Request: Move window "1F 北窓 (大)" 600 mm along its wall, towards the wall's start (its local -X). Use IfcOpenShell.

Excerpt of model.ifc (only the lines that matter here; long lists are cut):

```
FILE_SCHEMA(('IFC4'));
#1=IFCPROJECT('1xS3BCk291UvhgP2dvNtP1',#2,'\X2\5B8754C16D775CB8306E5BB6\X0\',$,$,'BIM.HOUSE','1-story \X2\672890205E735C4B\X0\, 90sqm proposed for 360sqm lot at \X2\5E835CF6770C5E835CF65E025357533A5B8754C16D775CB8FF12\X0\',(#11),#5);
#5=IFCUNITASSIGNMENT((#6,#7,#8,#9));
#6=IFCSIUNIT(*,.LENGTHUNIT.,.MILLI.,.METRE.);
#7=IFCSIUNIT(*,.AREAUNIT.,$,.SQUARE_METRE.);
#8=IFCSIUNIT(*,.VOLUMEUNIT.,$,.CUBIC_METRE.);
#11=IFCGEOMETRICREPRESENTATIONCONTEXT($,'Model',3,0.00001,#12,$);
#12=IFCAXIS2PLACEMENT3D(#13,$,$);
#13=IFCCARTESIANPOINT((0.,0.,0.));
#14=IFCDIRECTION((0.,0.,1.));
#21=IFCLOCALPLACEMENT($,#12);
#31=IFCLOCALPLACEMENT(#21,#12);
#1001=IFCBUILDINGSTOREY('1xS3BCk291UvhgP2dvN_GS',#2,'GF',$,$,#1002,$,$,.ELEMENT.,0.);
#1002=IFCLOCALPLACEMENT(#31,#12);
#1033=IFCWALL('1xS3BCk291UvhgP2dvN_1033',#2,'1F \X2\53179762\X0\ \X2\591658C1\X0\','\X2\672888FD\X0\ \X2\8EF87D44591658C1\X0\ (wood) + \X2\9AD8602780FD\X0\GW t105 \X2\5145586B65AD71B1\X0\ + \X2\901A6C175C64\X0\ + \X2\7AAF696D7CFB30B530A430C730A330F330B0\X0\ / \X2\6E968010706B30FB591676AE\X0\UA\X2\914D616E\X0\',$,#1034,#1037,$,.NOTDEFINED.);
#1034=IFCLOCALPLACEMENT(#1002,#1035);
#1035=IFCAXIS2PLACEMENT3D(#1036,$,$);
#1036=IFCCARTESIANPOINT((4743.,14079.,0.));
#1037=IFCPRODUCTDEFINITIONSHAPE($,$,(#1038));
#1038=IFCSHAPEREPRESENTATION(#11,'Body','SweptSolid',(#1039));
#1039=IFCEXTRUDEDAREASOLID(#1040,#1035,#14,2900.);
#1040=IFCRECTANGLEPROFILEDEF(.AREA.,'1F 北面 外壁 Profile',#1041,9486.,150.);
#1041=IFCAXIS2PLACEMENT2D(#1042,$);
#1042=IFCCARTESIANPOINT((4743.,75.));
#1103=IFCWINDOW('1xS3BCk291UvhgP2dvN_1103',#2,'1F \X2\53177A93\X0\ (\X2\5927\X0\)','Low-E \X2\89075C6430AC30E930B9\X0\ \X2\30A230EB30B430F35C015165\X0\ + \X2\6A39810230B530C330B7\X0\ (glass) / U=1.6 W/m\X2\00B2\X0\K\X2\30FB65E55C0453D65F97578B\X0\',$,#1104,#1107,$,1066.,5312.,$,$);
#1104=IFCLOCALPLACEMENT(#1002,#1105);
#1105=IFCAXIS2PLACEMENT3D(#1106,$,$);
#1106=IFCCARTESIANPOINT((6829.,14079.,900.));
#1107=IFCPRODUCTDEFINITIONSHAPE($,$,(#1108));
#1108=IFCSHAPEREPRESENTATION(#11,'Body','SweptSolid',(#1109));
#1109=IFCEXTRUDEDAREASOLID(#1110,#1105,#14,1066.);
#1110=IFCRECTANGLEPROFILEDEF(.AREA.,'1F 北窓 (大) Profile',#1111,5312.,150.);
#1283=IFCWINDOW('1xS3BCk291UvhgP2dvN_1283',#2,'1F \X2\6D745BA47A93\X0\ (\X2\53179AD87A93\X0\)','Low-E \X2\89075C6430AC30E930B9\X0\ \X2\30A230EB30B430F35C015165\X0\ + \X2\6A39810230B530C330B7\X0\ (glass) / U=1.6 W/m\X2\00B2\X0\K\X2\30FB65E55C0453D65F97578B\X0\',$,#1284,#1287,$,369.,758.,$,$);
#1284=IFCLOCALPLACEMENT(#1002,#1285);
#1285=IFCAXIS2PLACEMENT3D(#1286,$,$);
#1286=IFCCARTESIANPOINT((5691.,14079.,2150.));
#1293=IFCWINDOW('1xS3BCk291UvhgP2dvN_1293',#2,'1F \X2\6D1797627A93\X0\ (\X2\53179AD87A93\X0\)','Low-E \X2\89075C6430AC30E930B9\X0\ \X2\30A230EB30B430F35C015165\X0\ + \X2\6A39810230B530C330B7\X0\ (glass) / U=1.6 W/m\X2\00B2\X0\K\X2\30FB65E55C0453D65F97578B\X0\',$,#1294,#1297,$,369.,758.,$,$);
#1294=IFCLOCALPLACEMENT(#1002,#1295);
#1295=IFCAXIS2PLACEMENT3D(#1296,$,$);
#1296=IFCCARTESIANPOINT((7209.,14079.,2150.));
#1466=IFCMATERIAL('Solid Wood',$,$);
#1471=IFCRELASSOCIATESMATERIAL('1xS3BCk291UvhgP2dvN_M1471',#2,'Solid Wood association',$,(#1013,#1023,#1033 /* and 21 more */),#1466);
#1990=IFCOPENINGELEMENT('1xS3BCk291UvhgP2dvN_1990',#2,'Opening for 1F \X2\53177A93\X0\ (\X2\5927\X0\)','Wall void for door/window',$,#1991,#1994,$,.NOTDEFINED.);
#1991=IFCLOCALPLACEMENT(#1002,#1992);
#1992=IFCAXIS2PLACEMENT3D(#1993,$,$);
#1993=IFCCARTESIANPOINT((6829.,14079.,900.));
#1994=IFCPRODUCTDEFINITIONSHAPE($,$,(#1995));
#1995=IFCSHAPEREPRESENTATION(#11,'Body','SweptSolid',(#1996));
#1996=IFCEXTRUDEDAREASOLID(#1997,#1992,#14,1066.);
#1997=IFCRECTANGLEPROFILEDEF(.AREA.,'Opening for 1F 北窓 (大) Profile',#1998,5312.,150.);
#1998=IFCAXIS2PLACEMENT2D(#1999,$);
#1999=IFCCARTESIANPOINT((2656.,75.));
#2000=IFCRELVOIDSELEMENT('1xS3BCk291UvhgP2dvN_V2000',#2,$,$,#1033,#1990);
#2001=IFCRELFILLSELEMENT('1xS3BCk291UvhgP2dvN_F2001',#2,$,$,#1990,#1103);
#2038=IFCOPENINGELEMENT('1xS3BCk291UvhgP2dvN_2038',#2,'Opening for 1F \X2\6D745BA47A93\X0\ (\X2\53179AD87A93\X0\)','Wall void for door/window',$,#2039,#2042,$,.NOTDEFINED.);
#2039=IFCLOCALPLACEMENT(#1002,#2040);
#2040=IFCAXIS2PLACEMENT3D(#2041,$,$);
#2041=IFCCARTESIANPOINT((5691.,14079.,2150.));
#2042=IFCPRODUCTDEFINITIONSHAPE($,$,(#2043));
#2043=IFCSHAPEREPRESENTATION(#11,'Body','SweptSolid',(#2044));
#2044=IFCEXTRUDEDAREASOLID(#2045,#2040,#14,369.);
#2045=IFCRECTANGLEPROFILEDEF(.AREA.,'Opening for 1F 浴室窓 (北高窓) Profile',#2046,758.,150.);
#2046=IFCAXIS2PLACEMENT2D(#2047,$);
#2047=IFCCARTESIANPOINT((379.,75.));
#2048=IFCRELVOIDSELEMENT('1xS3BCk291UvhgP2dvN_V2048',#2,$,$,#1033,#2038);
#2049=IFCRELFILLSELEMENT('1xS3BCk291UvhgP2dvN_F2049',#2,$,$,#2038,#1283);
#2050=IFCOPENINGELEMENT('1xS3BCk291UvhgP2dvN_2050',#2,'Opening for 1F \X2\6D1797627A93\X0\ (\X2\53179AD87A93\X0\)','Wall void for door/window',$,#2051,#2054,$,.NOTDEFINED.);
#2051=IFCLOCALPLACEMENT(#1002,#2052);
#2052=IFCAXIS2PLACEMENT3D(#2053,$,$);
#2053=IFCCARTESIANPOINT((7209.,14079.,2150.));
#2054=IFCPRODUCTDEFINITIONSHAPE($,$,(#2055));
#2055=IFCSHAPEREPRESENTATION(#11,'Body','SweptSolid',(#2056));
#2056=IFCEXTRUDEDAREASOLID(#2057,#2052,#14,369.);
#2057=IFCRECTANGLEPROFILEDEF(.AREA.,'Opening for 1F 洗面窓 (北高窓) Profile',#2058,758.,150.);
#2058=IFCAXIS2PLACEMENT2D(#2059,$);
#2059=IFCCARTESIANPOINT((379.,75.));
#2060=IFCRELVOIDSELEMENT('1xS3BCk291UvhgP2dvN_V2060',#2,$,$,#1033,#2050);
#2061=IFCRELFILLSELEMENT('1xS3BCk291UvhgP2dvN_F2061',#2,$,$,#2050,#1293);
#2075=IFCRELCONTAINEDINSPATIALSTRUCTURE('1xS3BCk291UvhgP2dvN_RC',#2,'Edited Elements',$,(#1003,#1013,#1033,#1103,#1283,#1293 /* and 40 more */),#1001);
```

```python
import ifcopenshell
import ifcopenshell.api.geometry
import ifcopenshell.util.placement

model = ifcopenshell.open("model.ifc")

window = model.by_guid("1xS3BCk291UvhgP2dvN_1103")
opening = window.FillsVoids[0].RelatingOpeningElement
wall = opening.VoidsElements[0].RelatingBuildingElement

wall_matrix = ifcopenshell.util.placement.get_local_placement(wall.ObjectPlacement)
shift = wall_matrix[:3, 0] * -600.0
before = ifcopenshell.util.placement.get_local_placement(window.ObjectPlacement)[:3, 3].copy()

# The window is not placed relative to its opening, so move both.
for product in (opening, window):
    matrix = ifcopenshell.util.placement.get_local_placement(product.ObjectPlacement)
    matrix[:3, 3] += shift
    ifcopenshell.api.geometry.edit_object_placement(model, product=product, matrix=matrix, is_si=False)

after = ifcopenshell.util.placement.get_local_placement(window.ObjectPlacement)[:3, 3]
print("window moved by", (after - before).round(3) + 0.0)

model.write("model_edited.ifc")
```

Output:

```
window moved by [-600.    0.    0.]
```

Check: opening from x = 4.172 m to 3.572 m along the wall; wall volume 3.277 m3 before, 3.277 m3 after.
